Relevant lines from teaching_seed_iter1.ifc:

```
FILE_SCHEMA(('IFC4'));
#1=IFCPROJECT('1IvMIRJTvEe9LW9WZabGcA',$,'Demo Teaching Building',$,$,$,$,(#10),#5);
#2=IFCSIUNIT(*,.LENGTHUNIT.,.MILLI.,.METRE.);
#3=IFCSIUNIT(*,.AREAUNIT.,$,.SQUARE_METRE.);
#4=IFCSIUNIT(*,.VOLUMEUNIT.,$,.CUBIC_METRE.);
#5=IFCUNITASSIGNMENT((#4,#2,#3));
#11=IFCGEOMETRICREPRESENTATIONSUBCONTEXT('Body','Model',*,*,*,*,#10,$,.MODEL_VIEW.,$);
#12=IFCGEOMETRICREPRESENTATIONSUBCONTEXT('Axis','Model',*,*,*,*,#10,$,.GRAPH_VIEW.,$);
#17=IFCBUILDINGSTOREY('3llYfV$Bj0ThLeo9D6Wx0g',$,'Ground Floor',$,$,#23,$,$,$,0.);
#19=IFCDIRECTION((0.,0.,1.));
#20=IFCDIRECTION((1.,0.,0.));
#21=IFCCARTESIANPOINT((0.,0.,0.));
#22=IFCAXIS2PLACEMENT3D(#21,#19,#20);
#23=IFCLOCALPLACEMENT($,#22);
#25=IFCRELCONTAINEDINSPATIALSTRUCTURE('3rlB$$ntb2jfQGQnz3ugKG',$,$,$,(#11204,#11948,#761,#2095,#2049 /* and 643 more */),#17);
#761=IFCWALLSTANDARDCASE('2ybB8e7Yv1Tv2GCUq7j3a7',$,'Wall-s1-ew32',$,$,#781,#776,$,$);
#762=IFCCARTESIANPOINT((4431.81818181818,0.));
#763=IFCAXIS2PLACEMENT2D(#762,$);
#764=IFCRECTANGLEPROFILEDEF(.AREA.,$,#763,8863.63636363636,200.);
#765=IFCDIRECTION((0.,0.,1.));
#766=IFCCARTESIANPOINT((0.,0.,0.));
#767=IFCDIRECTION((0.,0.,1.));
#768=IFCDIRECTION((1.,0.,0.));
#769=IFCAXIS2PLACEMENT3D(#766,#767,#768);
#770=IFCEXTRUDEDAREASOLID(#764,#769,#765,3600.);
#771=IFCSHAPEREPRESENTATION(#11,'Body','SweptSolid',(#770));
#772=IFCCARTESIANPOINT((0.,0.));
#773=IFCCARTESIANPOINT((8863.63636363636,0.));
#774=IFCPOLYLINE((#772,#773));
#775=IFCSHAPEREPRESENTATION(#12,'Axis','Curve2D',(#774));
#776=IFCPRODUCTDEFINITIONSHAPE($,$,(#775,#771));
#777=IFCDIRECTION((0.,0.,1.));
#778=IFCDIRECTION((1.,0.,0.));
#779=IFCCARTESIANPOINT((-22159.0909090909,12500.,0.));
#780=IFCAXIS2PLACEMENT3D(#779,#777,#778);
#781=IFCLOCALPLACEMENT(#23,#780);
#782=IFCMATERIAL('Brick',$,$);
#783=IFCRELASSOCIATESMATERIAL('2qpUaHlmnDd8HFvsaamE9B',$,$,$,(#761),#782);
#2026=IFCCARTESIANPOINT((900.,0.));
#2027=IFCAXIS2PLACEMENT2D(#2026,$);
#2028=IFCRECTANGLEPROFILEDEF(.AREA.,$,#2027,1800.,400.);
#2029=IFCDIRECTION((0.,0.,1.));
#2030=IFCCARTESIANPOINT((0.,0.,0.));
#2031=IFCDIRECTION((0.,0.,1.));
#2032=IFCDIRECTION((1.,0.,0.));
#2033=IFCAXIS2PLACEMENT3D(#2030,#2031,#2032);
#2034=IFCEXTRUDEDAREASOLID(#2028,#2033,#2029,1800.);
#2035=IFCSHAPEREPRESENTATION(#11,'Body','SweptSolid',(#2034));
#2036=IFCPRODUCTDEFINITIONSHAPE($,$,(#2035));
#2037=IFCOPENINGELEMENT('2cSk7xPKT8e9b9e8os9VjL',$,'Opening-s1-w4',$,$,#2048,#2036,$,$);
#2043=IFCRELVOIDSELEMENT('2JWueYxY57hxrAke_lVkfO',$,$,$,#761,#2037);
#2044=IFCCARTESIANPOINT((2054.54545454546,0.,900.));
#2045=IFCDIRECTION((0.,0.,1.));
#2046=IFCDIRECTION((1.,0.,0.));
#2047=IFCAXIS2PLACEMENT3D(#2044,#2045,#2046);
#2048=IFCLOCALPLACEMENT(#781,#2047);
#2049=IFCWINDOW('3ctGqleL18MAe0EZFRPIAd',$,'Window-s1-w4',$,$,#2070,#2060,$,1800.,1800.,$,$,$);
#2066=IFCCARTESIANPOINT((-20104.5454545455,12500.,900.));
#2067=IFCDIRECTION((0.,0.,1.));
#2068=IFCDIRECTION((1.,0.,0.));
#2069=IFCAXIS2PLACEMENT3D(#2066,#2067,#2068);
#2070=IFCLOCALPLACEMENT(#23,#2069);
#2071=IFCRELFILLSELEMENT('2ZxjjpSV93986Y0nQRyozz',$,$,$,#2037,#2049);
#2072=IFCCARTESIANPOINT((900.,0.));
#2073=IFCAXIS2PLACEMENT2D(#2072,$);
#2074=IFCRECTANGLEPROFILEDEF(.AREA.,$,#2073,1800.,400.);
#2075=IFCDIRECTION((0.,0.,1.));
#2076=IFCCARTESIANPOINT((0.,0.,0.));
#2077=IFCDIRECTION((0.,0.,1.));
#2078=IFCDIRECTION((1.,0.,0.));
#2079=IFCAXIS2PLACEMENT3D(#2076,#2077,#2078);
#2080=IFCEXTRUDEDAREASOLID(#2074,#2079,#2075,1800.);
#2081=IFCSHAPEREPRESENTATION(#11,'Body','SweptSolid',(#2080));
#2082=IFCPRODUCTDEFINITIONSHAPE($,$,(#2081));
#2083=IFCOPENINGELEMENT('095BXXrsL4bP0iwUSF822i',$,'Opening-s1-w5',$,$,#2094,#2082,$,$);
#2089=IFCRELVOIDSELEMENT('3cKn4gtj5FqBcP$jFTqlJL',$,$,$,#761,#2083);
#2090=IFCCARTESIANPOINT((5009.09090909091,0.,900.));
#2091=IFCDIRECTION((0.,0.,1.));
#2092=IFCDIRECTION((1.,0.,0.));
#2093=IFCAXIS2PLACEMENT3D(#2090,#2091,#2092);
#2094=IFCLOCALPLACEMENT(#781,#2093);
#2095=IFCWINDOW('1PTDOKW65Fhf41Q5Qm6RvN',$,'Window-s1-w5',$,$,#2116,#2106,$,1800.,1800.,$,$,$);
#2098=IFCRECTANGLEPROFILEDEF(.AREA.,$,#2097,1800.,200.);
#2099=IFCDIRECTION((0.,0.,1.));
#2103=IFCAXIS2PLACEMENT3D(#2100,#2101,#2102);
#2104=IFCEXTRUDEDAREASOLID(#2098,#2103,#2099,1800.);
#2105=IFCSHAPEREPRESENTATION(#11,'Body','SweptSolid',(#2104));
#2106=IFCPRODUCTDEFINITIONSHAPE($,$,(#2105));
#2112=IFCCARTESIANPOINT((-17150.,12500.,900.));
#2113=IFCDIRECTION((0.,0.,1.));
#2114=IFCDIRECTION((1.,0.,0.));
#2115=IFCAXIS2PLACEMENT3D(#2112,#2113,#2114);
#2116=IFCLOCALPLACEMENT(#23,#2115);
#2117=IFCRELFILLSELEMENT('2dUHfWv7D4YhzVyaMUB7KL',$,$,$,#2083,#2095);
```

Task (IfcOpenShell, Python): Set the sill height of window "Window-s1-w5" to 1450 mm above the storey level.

```python
import numpy as np
import ifcopenshell
import ifcopenshell.api.geometry
import ifcopenshell.geom
import ifcopenshell.util.element
import ifcopenshell.util.placement
import ifcopenshell.util.shape
import ifcopenshell.util.unit

model = ifcopenshell.open("teaching_seed_iter1.ifc")
unit_scale = ifcopenshell.util.unit.calculate_unit_scale(model)

window = model.by_id(2095)
opening = window.FillsVoids[0].RelatingOpeningElement
storey = ifcopenshell.util.element.get_container(window, ifc_class="IfcBuildingStorey")
level = ifcopenshell.util.placement.get_local_placement(storey.ObjectPlacement)[2, 3]

# The opening's origin need not be at the sill, so measure its lowest point.
shape = ifcopenshell.geom.create_shape(ifcopenshell.geom.settings(), opening)
bottom = ifcopenshell.util.shape.get_shape_bottom_elevation(shape, shape.geometry) / unit_scale
dz = level + 1450.0 - bottom

shift = np.array([0.0, 0.0, dz])
# The window is not placed relative to its opening, so move both.
for product in (opening, window):
    matrix = ifcopenshell.util.placement.get_local_placement(product.ObjectPlacement)
    matrix[:3, 3] += shift
    ifcopenshell.api.geometry.edit_object_placement(model, product=product, matrix=matrix, is_si=False)

print(f"moved by {dz * unit_scale:+.3f} m")

model.write("teaching_seed_iter1_v2.ifc")
```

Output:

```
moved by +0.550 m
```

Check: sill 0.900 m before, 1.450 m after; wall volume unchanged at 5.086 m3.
